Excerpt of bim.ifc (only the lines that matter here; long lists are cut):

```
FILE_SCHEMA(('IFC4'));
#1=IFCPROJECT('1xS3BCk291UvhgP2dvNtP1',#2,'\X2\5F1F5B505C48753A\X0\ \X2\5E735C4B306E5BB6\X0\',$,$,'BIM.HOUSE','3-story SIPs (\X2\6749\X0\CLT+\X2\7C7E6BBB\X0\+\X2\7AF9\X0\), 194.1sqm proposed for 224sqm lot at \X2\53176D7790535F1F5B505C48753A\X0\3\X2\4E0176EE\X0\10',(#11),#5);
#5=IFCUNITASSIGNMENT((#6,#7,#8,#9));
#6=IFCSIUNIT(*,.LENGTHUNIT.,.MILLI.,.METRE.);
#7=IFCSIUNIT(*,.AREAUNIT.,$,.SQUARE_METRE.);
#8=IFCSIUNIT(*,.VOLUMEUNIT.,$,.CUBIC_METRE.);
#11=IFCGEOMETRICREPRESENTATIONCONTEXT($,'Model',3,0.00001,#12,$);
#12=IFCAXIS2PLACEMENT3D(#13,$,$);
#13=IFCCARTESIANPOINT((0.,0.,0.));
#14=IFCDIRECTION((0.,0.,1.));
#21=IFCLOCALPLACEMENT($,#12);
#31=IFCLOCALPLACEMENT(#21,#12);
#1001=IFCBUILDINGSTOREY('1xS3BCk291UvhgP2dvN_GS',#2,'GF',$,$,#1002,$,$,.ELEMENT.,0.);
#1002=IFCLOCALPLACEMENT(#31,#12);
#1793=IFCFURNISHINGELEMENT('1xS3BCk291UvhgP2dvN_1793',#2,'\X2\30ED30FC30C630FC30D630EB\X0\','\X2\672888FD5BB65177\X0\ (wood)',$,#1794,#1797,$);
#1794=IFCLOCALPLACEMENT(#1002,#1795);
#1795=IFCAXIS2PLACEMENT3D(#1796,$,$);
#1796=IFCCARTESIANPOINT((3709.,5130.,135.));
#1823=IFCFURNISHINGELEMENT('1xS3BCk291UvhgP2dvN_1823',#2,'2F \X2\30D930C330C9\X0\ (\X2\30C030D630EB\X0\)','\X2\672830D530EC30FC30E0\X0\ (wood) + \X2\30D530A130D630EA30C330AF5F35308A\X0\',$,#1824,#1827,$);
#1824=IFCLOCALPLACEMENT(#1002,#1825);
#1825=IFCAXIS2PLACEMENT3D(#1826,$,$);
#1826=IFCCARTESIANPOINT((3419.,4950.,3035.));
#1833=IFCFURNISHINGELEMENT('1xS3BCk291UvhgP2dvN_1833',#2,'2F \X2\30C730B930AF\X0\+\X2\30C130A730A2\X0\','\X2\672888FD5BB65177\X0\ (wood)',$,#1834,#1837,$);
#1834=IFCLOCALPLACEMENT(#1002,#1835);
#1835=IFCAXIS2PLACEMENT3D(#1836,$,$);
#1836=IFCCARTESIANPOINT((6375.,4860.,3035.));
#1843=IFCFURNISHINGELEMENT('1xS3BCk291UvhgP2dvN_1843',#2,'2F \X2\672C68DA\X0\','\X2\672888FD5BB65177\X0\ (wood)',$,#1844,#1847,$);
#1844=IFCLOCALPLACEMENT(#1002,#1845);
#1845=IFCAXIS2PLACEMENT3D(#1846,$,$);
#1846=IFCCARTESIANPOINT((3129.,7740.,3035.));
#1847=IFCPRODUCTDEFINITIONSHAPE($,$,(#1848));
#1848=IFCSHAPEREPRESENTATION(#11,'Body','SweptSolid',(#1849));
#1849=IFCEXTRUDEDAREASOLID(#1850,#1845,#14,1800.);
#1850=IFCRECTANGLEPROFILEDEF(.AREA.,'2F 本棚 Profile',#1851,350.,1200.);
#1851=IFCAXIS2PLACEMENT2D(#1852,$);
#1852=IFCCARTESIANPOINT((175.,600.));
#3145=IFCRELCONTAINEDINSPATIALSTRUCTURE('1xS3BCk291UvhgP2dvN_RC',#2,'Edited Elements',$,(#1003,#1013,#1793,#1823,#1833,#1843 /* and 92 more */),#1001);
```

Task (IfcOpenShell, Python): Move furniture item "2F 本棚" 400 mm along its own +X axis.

```python
import ifcopenshell
import ifcopenshell.api.geometry
import ifcopenshell.util.placement
import ifcopenshell.util.unit

model = ifcopenshell.open("bim.ifc")
unit_scale = ifcopenshell.util.unit.calculate_unit_scale(model)

item = model.by_guid("1xS3BCk291UvhgP2dvN_1843")
matrix = ifcopenshell.util.placement.get_local_placement(item.ObjectPlacement)
matrix[:3, 3] += matrix[:3, 0] * 0.4 / unit_scale
ifcopenshell.api.geometry.edit_object_placement(model, product=item, matrix=matrix, is_si=False)

print(ifcopenshell.util.placement.get_local_placement(item.ObjectPlacement).round(3) + 0.0)

model.write("bim_v2.ifc")
```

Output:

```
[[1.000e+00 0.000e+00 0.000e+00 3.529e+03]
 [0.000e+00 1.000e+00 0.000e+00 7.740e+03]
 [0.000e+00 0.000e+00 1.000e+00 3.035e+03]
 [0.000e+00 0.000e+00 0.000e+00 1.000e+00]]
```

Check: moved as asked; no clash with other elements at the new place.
